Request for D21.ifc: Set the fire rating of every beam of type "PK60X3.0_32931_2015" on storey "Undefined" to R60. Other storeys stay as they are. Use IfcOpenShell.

First a look at what the model holds.

```python
import ifcopenshell
import ifcopenshell.util.element

model = ifcopenshell.open("D21.ifc")
print(model.schema)
storey = next(s for s in model.by_type("IfcBuildingStorey") if s.Name == "Undefined")
beams = [e for e in ifcopenshell.util.element.get_decomposition(storey) if e.is_a("IfcBeam")]
seen = {}
for e in beams:
    element_type = ifcopenshell.util.element.get_type(e)
    key = (element_type.Name if element_type != e and element_type else None, ifcopenshell.util.element.get_pset(e, "Pset_BeamCommon", "FireRating"))
    seen[key] = seen.get(key, 0) + 1
for (name, value), count in sorted(seen.items(), key=str):
    print(count, "x", name, "|", value)
```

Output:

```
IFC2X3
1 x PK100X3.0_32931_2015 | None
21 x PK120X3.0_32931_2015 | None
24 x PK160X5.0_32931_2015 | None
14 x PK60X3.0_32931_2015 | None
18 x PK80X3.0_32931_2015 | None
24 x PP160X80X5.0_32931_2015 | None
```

```python
import ifcopenshell
import ifcopenshell.api.pset
import ifcopenshell.util.element

model = ifcopenshell.open("D21.ifc")

storey = next(s for s in model.by_type("IfcBuildingStorey") if s.Name == "Undefined")
beams = [e for e in ifcopenshell.util.element.get_decomposition(storey) if e.is_a("IfcBeam")]

count = 0
for e in beams:
    element_type = ifcopenshell.util.element.get_type(e)
    if element_type in (None, e) or element_type.Name != "PK60X3.0_32931_2015":
        continue
    found = ifcopenshell.util.element.get_pset(e, "Pset_BeamCommon", should_inherit=False)
    if found:
        pset = model.by_id(found["id"])
        if len(ifcopenshell.util.element.get_elements_by_pset(pset)) > 1:
            pset = ifcopenshell.api.pset.unshare_pset(model, products=[e], pset=pset)[0]
    else:
        pset = ifcopenshell.api.pset.add_pset(model, product=e, name="Pset_BeamCommon")
    ifcopenshell.api.pset.edit_pset(model, pset=pset, properties={"FireRating": "R60"})
    count += 1

print(count, "beams updated")

model.write("D21-out.ifc")
```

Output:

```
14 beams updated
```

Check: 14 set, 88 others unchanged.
